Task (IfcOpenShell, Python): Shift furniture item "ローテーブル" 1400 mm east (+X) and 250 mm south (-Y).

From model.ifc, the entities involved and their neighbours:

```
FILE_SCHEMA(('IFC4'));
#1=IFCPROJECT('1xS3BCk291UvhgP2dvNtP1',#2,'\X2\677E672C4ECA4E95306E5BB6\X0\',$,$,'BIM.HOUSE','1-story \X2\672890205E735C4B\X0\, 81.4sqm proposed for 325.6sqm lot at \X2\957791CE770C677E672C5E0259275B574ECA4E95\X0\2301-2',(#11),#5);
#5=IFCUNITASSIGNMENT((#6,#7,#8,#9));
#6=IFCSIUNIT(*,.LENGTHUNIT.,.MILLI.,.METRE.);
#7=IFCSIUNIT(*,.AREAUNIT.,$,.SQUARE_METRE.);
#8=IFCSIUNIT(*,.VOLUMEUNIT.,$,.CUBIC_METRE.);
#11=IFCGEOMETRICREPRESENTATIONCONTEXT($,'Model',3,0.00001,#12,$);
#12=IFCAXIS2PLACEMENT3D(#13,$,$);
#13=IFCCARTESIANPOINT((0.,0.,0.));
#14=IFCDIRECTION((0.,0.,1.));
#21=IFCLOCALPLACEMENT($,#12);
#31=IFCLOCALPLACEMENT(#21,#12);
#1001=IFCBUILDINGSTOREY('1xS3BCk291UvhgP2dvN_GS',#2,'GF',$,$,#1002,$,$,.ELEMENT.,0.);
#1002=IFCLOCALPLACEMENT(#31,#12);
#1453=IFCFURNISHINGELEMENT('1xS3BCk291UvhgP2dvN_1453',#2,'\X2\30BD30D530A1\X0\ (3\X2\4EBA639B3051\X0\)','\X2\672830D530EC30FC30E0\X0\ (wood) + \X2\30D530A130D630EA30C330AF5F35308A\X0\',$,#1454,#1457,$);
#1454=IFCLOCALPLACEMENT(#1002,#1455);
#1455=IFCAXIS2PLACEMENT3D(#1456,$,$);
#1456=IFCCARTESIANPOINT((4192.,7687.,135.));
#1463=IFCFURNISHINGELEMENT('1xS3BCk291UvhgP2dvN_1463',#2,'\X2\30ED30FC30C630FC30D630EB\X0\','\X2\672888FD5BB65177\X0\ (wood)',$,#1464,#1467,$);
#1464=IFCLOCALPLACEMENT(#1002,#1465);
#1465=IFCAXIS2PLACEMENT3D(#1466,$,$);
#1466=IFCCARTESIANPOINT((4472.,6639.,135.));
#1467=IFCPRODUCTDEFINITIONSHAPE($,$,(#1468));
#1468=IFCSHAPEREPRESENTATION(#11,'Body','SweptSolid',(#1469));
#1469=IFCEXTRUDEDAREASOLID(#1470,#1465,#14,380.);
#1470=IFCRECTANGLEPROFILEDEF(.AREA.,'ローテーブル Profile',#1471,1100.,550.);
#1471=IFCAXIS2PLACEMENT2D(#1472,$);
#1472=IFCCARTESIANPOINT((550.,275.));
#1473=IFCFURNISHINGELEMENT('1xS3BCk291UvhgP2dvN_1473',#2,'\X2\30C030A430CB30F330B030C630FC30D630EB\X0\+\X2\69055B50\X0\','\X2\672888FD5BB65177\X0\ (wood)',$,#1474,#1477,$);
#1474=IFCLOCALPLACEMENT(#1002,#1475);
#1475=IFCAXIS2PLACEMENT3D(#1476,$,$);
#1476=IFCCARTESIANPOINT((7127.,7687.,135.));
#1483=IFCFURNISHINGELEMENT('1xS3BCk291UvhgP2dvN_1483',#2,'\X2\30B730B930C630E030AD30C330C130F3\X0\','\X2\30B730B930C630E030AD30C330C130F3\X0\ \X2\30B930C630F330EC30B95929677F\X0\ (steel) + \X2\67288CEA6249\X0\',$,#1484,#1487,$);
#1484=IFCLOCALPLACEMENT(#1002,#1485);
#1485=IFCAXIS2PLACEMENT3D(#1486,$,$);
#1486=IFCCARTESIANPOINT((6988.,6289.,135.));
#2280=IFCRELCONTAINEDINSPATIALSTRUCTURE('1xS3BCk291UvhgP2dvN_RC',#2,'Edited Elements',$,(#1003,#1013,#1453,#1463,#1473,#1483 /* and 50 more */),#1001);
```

```python
import ifcopenshell
import ifcopenshell.api.geometry
import ifcopenshell.util.placement

model = ifcopenshell.open("model.ifc")

item = model.by_guid("1xS3BCk291UvhgP2dvN_1463")
matrix = ifcopenshell.util.placement.get_local_placement(item.ObjectPlacement)
matrix[0, 3] += 1400.0
matrix[1, 3] -= 250.0
ifcopenshell.api.geometry.edit_object_placement(model, product=item, matrix=matrix, is_si=False)

print(ifcopenshell.util.placement.get_local_placement(item.ObjectPlacement).round(3) + 0.0)

model.write("model_updated.ifc")
```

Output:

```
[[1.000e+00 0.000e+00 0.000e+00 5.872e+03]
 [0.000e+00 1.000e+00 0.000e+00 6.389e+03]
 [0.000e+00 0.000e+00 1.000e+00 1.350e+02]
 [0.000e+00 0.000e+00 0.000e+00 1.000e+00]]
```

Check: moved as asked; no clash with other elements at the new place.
